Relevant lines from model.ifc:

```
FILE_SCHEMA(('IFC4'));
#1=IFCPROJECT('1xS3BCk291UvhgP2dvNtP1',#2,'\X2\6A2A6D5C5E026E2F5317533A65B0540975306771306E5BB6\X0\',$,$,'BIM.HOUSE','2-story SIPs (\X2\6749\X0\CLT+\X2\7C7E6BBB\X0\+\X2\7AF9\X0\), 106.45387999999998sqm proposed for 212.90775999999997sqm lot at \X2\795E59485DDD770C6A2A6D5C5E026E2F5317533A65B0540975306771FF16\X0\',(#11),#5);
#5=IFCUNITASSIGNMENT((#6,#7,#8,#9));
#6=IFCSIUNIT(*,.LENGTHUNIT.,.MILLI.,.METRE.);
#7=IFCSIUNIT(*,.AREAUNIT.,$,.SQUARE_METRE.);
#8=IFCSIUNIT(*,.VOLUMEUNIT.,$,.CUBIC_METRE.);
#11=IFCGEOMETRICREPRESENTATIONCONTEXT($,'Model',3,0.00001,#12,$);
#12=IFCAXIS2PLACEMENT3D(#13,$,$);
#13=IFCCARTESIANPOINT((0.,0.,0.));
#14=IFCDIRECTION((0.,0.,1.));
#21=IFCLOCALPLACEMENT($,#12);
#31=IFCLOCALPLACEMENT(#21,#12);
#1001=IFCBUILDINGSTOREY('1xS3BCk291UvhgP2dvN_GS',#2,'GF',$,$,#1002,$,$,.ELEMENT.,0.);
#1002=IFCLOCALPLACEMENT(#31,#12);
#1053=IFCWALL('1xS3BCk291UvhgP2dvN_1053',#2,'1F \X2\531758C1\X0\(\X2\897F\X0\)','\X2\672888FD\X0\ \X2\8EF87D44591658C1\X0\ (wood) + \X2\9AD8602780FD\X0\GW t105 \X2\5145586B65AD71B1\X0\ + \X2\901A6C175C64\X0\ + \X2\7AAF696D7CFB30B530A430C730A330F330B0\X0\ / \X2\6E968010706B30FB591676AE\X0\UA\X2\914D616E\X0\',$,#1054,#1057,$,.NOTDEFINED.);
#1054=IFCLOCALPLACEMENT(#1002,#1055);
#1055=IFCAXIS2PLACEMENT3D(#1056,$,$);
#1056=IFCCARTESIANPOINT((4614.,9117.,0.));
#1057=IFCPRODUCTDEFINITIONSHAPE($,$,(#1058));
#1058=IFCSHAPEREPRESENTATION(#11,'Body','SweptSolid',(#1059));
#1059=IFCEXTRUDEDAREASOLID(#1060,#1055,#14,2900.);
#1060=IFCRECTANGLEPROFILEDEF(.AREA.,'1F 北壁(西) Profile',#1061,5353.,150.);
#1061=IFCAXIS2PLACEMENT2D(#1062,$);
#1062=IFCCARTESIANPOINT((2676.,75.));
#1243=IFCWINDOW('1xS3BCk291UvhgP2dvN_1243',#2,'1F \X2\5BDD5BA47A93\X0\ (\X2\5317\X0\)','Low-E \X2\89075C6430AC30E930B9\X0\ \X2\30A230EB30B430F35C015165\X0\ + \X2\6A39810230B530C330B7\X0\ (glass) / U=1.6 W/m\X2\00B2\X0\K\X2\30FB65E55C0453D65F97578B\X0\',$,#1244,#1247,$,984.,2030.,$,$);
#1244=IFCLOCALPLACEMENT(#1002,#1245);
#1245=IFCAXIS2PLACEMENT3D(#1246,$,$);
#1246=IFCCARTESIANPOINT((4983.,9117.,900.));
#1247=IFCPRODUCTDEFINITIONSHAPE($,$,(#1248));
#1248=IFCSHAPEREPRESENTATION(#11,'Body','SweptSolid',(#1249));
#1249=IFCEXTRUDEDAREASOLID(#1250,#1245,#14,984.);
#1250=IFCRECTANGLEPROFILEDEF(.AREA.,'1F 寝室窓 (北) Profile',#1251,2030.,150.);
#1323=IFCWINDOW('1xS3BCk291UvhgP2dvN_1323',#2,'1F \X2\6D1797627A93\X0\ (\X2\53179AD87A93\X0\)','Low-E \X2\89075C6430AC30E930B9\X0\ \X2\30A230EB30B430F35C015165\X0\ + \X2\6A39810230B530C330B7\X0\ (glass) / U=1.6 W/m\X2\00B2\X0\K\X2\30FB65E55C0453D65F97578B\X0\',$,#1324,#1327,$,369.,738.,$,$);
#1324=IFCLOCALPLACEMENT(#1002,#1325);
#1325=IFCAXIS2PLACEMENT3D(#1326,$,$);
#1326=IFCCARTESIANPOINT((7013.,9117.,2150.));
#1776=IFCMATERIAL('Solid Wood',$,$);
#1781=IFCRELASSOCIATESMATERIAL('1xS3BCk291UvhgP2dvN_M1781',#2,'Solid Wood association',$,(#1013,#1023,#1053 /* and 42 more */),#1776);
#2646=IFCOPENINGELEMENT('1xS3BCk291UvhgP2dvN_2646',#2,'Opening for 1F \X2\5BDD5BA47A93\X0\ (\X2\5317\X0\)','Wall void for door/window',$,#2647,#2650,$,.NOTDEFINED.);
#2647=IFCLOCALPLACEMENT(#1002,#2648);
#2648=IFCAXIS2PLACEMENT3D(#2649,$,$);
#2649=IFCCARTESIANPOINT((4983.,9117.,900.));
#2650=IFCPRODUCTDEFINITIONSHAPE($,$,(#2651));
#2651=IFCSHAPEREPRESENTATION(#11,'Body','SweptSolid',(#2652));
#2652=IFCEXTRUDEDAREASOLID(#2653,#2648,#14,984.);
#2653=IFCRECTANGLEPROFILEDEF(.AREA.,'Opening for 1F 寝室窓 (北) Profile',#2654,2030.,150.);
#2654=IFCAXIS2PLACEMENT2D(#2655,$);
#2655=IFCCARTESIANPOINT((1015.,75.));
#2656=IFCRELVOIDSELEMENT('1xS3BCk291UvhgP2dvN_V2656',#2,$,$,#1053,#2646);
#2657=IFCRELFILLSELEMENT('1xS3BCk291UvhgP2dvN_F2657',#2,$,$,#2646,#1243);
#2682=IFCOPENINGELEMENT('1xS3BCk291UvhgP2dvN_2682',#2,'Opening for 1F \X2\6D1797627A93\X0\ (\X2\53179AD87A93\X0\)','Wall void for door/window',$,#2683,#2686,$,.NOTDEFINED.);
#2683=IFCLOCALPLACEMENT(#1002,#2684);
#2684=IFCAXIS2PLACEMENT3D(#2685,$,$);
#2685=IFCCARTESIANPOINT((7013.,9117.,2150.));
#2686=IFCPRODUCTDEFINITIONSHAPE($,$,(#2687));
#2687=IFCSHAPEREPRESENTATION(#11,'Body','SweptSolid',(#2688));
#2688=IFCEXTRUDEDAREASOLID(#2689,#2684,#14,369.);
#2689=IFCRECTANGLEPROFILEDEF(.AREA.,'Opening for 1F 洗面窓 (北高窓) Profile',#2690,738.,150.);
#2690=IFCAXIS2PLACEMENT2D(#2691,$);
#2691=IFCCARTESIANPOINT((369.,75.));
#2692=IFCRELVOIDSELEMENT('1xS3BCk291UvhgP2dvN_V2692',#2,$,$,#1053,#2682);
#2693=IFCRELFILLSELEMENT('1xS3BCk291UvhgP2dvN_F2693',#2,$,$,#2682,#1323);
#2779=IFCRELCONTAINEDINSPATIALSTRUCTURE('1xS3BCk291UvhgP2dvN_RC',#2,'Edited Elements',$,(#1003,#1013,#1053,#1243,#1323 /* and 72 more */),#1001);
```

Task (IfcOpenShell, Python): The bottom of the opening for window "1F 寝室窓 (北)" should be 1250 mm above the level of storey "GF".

```python
import numpy as np
import ifcopenshell
import ifcopenshell.api.geometry
import ifcopenshell.geom
import ifcopenshell.util.element
import ifcopenshell.util.placement
import ifcopenshell.util.shape
import ifcopenshell.util.unit

model = ifcopenshell.open("model.ifc")
unit_scale = ifcopenshell.util.unit.calculate_unit_scale(model)

window = model.by_id(1243)
opening = window.FillsVoids[0].RelatingOpeningElement
storey = ifcopenshell.util.element.get_container(window, ifc_class="IfcBuildingStorey")
level = ifcopenshell.util.placement.get_local_placement(storey.ObjectPlacement)[2, 3]

# The opening's origin need not be at the sill, so measure its lowest point.
shape = ifcopenshell.geom.create_shape(ifcopenshell.geom.settings(), opening)
bottom = ifcopenshell.util.shape.get_shape_bottom_elevation(shape, shape.geometry) / unit_scale
dz = level + 1.25 / unit_scale - bottom

shift = np.array([0.0, 0.0, dz])
# The window is not placed relative to its opening, so move both.
for product in (opening, window):
    matrix = ifcopenshell.util.placement.get_local_placement(product.ObjectPlacement)
    matrix[:3, 3] += shift
    ifcopenshell.api.geometry.edit_object_placement(model, product=product, matrix=matrix, is_si=False)

print(f"moved by {dz * unit_scale:+.3f} m")

model.write("model_edited.ifc")
```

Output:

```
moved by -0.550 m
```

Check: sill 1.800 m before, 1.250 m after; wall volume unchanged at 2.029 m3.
